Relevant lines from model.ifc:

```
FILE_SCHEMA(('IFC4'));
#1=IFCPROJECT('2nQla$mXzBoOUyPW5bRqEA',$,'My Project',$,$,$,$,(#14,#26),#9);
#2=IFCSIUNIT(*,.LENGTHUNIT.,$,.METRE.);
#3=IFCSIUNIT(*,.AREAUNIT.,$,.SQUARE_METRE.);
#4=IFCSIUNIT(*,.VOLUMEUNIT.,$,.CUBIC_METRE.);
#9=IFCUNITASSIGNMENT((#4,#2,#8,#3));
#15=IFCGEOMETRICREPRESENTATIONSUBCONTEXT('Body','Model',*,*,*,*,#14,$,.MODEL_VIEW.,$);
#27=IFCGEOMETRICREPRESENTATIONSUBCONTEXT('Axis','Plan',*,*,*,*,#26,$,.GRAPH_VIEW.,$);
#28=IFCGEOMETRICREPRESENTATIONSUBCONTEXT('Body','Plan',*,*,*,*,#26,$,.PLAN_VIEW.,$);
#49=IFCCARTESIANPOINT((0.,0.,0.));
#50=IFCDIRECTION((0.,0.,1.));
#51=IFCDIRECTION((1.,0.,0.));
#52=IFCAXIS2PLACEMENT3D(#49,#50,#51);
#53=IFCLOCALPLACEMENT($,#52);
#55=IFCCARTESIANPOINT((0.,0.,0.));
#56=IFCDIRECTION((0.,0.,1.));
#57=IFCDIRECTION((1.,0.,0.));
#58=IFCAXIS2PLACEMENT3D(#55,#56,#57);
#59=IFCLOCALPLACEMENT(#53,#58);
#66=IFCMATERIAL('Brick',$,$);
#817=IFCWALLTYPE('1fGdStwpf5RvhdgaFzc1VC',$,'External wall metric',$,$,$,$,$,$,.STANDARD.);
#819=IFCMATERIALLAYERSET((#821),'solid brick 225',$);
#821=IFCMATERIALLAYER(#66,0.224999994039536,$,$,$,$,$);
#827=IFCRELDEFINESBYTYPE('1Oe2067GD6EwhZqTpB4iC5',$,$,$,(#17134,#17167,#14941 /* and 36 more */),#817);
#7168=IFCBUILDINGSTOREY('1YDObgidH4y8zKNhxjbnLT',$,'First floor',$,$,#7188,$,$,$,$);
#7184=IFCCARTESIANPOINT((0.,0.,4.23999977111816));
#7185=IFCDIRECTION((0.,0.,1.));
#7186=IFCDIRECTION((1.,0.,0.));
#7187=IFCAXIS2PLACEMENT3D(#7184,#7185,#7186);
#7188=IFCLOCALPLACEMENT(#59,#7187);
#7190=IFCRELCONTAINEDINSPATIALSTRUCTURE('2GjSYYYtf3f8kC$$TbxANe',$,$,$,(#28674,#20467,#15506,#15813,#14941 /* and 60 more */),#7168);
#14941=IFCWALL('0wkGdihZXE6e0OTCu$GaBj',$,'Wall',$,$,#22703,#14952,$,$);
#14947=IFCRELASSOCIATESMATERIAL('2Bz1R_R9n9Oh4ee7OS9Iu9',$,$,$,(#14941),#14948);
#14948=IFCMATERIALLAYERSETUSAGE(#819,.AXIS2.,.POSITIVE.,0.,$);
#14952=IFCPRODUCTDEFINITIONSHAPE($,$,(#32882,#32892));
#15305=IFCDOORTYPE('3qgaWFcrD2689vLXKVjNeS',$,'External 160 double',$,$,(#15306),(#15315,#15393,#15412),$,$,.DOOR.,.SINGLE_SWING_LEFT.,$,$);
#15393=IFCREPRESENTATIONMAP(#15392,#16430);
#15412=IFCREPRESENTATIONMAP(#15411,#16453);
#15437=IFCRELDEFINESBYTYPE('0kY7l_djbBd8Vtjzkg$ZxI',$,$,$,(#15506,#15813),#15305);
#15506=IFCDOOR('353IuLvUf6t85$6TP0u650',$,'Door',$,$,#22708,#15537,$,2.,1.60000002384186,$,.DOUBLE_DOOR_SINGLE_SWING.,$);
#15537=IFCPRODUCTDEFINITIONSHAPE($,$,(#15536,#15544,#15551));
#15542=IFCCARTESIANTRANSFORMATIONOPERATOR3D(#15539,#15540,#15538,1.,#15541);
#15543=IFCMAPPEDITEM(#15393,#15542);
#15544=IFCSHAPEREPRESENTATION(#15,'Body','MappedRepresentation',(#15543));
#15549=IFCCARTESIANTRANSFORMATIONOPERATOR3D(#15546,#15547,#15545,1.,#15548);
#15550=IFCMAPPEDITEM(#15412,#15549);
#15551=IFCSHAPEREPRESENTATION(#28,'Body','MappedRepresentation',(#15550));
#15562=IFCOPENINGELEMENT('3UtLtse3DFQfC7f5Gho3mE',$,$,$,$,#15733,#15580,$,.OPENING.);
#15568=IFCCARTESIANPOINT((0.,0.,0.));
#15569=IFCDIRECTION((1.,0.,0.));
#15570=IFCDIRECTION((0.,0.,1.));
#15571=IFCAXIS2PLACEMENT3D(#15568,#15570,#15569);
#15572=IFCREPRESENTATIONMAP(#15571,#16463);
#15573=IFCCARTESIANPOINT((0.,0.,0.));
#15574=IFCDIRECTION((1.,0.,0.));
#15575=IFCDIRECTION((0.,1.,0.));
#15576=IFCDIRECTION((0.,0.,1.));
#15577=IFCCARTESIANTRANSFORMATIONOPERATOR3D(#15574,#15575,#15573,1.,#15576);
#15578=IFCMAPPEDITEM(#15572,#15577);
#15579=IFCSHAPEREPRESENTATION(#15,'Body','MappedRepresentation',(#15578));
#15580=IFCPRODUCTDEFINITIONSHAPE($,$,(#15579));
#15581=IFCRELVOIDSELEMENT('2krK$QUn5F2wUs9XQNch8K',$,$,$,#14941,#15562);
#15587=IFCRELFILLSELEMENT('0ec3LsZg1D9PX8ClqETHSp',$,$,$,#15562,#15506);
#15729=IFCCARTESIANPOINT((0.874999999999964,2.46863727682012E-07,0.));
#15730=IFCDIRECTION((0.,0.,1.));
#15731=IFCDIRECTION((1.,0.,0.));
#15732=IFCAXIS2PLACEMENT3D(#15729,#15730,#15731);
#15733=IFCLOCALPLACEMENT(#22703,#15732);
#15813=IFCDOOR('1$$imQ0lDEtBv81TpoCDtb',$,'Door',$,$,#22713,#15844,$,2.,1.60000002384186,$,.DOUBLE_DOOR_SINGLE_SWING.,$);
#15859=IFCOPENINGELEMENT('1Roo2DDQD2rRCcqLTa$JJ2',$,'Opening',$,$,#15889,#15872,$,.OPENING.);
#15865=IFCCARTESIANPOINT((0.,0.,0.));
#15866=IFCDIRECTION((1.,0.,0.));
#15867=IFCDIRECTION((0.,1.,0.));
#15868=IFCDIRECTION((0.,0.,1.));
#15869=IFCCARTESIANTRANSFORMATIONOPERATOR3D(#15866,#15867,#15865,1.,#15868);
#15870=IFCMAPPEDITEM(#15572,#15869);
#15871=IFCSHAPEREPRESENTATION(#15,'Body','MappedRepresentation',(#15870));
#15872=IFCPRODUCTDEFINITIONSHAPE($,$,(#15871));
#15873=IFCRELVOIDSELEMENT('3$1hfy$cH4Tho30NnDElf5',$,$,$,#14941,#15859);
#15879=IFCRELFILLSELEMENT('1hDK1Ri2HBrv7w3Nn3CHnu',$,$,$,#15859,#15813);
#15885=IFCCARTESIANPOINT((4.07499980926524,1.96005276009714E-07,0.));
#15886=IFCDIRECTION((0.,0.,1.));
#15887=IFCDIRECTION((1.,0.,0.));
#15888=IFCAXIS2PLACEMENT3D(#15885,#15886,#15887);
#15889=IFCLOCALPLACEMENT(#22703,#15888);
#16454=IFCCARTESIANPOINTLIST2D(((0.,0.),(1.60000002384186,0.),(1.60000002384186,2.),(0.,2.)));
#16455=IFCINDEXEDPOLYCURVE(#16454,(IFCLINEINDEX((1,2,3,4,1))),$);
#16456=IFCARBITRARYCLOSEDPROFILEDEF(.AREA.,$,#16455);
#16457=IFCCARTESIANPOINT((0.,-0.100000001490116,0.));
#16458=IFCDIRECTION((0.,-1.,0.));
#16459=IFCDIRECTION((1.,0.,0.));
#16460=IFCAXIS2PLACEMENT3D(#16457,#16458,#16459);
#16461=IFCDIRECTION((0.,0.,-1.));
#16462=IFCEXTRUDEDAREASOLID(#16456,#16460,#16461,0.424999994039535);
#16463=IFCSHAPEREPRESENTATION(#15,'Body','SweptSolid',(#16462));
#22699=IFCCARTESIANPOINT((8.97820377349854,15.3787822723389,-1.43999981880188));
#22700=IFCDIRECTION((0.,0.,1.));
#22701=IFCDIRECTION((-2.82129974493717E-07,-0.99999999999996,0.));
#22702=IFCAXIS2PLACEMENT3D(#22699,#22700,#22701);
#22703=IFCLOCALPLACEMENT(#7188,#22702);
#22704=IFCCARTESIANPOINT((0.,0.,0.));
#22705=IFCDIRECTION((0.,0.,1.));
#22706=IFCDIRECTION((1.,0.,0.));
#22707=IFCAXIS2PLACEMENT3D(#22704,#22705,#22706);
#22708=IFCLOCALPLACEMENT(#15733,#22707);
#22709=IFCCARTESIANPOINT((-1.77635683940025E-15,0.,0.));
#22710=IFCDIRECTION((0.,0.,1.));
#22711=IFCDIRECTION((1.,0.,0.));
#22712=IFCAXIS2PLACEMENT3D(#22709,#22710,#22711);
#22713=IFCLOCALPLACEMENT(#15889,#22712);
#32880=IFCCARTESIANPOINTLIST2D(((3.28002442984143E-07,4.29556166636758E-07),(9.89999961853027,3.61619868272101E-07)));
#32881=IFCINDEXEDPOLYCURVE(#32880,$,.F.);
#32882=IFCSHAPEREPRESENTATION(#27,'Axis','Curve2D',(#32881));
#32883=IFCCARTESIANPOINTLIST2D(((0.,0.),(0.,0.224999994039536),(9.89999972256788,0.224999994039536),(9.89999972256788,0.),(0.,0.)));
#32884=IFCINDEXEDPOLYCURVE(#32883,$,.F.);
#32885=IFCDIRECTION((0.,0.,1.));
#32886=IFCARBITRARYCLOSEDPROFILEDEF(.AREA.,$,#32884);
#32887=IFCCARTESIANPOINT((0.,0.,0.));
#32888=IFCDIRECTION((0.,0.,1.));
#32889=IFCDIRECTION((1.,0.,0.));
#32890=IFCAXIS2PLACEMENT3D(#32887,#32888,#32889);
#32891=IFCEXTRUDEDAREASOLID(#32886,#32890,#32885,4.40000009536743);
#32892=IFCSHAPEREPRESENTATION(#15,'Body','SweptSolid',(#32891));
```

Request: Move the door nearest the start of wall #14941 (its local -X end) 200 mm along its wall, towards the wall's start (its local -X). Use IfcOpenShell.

```python
import ifcopenshell
import ifcopenshell.api.geometry
import ifcopenshell.util.placement
import ifcopenshell.util.unit

model = ifcopenshell.open("model.ifc")
unit_scale = ifcopenshell.util.unit.calculate_unit_scale(model)

door = model.by_id(15506)
opening = door.FillsVoids[0].RelatingOpeningElement
wall = opening.VoidsElements[0].RelatingBuildingElement

wall_matrix = ifcopenshell.util.placement.get_local_placement(wall.ObjectPlacement)
shift = wall_matrix[:3, 0] * -0.2 / unit_scale
before = ifcopenshell.util.placement.get_local_placement(door.ObjectPlacement)[:3, 3].copy()

# The door is placed relative to its opening, so it follows when the opening moves.
matrix = ifcopenshell.util.placement.get_local_placement(opening.ObjectPlacement)
matrix[:3, 3] += shift
ifcopenshell.api.geometry.edit_object_placement(
    model, product=opening, matrix=matrix, is_si=False, should_transform_children=True
)

after = ifcopenshell.util.placement.get_local_placement(door.ObjectPlacement)[:3, 3]
print("door moved by", (after - before).round(3) + 0.0)

model.write("model_rev.ifc")
```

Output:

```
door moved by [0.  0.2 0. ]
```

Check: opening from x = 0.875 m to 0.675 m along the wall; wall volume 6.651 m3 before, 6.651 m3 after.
